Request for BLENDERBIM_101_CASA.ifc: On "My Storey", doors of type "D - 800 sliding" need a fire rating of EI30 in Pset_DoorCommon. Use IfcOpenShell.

First a look at what the model holds.

```python
import ifcopenshell
import ifcopenshell.util.element

model = ifcopenshell.open("BLENDERBIM_101_CASA.ifc")
print(model.schema)
storey = next(s for s in model.by_type("IfcBuildingStorey") if s.Name == "My Storey")
doors = [e for e in ifcopenshell.util.element.get_decomposition(storey) if e.is_a("IfcDoor")]
seen = {}
for e in doors:
    element_type = ifcopenshell.util.element.get_type(e)
    key = (element_type.Name if element_type != e and element_type else None, ifcopenshell.util.element.get_pset(e, "Pset_DoorCommon", "FireRating"))
    seen[key] = seen.get(key, 0) + 1
for (name, value), count in sorted(seen.items(), key=str):
    print(count, "x", name, "|", value)
```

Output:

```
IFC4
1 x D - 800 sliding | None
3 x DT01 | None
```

```python
import ifcopenshell
import ifcopenshell.api.pset
import ifcopenshell.util.element

model = ifcopenshell.open("BLENDERBIM_101_CASA.ifc")

storey = next(s for s in model.by_type("IfcBuildingStorey") if s.Name == "My Storey")
doors = [e for e in ifcopenshell.util.element.get_decomposition(storey) if e.is_a("IfcDoor")]

count = 0
for e in doors:
    element_type = ifcopenshell.util.element.get_type(e)
    if element_type in (None, e) or element_type.Name != "D - 800 sliding":
        continue
    # add_pset returns the element's existing set when there is one.
    pset = ifcopenshell.api.pset.add_pset(model, product=e, name="Pset_DoorCommon")
    ifcopenshell.api.pset.edit_pset(model, pset=pset, properties={"FireRating": "EI30"})
    count += 1

print(count, "doors updated")

model.write("BLENDERBIM_101_CASA_rev.ifc")
```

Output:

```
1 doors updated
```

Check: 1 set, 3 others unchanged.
